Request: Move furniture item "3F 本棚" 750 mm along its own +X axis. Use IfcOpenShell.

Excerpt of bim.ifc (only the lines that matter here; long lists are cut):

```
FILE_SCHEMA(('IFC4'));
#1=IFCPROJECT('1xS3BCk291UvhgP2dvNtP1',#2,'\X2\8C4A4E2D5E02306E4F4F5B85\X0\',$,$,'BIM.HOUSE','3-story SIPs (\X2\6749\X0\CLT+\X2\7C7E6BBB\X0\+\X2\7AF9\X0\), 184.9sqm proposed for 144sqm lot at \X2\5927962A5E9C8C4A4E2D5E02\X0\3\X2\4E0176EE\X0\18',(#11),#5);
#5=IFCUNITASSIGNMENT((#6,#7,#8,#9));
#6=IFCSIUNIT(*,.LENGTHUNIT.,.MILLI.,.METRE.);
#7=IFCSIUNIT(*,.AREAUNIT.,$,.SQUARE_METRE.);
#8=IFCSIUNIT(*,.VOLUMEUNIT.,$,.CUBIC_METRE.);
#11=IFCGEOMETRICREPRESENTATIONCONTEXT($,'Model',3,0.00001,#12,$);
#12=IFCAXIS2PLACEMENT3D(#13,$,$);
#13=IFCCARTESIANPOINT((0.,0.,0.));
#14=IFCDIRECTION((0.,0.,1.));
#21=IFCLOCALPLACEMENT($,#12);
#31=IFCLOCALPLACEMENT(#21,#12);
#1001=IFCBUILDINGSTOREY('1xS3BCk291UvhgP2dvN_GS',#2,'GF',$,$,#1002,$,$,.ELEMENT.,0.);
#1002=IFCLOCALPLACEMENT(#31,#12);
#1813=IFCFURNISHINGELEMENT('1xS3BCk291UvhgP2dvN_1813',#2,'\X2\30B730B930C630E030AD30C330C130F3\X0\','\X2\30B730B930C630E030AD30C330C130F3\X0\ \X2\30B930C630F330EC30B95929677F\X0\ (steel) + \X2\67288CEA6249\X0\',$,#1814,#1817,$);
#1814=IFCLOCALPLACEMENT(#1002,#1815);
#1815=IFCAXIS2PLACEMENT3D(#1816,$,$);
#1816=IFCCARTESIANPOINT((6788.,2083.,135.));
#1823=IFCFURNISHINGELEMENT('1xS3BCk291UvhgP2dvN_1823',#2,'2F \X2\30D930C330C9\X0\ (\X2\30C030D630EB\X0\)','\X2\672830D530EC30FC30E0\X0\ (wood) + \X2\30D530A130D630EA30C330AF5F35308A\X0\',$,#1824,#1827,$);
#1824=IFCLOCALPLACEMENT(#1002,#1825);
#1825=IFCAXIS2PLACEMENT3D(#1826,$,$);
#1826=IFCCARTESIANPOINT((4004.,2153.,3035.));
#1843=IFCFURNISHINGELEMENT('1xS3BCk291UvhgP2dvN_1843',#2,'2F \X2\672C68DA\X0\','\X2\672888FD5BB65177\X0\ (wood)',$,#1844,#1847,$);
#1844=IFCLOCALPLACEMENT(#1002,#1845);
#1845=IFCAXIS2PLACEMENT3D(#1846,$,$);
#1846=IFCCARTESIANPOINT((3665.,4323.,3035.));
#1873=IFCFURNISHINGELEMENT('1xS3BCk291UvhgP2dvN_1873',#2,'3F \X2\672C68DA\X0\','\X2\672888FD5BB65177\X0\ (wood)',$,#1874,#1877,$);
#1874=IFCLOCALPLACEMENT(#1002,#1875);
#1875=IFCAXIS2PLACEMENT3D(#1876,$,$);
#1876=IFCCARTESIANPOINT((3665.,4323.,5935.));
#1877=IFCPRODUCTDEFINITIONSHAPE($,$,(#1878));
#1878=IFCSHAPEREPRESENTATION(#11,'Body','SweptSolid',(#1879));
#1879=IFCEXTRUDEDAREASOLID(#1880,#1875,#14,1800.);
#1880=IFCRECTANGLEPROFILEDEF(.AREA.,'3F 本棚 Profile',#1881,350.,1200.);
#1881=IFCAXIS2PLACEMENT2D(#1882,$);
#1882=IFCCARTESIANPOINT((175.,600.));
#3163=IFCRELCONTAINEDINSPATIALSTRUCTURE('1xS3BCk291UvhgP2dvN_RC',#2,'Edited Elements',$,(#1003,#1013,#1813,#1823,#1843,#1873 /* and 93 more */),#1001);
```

```python
import ifcopenshell
import ifcopenshell.api.geometry
import ifcopenshell.util.placement
import ifcopenshell.util.unit

model = ifcopenshell.open("bim.ifc")
unit_scale = ifcopenshell.util.unit.calculate_unit_scale(model)

item = model.by_id(1873)
matrix = ifcopenshell.util.placement.get_local_placement(item.ObjectPlacement)
matrix[:3, 3] += matrix[:3, 0] * 0.75 / unit_scale
ifcopenshell.api.geometry.edit_object_placement(model, product=item, matrix=matrix, is_si=False)

print(ifcopenshell.util.placement.get_local_placement(item.ObjectPlacement).round(3) + 0.0)

model.write("bim_rev.ifc")
```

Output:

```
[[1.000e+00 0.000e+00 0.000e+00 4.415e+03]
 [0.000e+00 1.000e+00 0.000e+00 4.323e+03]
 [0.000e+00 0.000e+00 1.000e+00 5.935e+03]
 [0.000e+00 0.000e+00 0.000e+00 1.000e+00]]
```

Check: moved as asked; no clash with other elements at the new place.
